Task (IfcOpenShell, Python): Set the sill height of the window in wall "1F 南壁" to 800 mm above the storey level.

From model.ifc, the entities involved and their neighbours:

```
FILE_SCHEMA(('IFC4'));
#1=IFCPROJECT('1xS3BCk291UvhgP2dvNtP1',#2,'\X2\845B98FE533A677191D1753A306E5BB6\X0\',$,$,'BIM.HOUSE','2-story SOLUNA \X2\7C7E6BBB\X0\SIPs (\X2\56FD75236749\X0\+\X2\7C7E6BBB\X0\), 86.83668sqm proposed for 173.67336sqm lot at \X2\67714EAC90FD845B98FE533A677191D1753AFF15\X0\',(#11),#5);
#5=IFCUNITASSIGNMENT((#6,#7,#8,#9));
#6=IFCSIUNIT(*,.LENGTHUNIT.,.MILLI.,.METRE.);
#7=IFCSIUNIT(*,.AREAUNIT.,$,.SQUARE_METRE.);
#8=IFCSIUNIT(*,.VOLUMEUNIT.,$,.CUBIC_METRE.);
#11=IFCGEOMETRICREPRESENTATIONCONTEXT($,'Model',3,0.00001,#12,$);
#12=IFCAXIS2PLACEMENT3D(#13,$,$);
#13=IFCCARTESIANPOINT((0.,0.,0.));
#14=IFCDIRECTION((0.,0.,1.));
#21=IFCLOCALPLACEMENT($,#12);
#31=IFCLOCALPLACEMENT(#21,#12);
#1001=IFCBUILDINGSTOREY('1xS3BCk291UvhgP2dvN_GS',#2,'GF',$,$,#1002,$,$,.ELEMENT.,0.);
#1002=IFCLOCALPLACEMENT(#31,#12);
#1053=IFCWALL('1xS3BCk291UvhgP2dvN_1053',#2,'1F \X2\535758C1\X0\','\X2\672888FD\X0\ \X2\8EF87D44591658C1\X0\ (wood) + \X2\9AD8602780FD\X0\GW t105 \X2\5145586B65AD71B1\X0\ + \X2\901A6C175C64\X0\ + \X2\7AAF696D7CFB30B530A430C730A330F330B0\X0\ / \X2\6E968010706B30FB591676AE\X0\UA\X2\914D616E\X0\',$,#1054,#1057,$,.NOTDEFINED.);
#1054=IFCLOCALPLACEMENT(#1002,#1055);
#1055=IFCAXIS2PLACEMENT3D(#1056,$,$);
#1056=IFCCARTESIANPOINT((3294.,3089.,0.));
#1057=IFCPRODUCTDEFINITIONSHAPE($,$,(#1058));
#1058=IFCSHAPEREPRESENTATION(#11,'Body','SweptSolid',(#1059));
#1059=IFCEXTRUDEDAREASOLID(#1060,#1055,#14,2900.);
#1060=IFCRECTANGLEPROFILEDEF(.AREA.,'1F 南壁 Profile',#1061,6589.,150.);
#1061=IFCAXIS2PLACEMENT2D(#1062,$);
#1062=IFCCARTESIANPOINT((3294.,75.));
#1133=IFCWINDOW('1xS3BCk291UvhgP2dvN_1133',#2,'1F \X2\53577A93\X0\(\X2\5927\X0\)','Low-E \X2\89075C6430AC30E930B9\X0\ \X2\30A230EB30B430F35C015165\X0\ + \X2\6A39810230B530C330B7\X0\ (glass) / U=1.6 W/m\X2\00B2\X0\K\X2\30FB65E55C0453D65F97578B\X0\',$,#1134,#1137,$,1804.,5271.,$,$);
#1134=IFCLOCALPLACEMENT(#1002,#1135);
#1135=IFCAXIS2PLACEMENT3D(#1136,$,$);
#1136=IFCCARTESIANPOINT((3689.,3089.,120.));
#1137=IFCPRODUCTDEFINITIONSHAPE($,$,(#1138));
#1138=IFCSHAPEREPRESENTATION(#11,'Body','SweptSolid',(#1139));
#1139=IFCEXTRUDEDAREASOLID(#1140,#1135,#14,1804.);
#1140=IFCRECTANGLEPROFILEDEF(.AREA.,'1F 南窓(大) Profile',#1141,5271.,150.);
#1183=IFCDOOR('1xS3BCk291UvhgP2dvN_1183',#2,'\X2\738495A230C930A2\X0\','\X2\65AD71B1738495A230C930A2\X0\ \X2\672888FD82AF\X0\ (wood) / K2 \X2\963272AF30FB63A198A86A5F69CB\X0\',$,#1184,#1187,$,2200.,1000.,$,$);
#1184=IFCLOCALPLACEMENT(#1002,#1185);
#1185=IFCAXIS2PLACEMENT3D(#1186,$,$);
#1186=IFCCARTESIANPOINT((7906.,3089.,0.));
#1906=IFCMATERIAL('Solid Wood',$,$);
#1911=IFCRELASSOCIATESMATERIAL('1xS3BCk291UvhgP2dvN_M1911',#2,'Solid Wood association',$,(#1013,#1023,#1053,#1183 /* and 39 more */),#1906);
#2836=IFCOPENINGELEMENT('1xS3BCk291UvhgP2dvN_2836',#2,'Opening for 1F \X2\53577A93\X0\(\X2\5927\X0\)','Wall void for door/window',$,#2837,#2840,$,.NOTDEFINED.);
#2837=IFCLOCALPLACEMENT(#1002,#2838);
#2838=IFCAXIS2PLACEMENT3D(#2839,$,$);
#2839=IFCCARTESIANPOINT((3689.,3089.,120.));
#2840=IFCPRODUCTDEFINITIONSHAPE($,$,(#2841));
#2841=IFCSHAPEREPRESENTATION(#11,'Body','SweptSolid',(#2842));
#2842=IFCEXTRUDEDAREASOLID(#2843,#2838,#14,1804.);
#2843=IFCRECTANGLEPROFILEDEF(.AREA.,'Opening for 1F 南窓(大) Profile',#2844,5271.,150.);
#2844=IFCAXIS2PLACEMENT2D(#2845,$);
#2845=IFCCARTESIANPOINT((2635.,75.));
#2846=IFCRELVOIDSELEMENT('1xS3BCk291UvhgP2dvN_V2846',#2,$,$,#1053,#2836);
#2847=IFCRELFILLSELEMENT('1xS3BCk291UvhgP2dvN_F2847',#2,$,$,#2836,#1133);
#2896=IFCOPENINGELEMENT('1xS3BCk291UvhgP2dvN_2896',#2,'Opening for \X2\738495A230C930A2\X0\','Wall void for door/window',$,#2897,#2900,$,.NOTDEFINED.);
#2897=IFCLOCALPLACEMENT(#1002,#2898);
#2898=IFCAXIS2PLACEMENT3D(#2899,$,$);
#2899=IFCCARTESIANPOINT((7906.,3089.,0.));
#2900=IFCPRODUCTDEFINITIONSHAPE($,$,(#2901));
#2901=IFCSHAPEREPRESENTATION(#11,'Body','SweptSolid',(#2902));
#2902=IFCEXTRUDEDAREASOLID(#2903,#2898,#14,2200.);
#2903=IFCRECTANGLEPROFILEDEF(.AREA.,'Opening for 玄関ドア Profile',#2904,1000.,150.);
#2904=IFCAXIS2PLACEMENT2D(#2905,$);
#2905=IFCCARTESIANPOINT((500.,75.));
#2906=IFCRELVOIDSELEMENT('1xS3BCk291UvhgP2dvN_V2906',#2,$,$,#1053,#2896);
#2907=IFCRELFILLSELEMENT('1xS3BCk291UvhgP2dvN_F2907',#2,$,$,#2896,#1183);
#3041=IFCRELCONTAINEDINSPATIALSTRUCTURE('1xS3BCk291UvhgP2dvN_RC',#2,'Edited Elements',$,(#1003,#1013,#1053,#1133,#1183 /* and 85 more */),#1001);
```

```python
import numpy as np
import ifcopenshell
import ifcopenshell.api.geometry
import ifcopenshell.geom
import ifcopenshell.util.element
import ifcopenshell.util.placement
import ifcopenshell.util.shape
import ifcopenshell.util.unit

model = ifcopenshell.open("model.ifc")
unit_scale = ifcopenshell.util.unit.calculate_unit_scale(model)

window = model.by_guid("1xS3BCk291UvhgP2dvN_1133")
opening = window.FillsVoids[0].RelatingOpeningElement
storey = ifcopenshell.util.element.get_container(window, ifc_class="IfcBuildingStorey")
level = ifcopenshell.util.placement.get_local_placement(storey.ObjectPlacement)[2, 3]

# The opening's origin need not be at the sill, so measure its lowest point.
shape = ifcopenshell.geom.create_shape(ifcopenshell.geom.settings(), opening)
bottom = ifcopenshell.util.shape.get_shape_bottom_elevation(shape, shape.geometry) / unit_scale
dz = level + 0.8 / unit_scale - bottom

shift = np.array([0.0, 0.0, dz])
# The window is not placed relative to its opening, so move both.
for product in (opening, window):
    matrix = ifcopenshell.util.placement.get_local_placement(product.ObjectPlacement)
    matrix[:3, 3] += shift
    ifcopenshell.api.geometry.edit_object_placement(model, product=product, matrix=matrix, is_si=False)

print(f"moved by {dz * unit_scale:+.3f} m")

model.write("model_v2.ifc")
```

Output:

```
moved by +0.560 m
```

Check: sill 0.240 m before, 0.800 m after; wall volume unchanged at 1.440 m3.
